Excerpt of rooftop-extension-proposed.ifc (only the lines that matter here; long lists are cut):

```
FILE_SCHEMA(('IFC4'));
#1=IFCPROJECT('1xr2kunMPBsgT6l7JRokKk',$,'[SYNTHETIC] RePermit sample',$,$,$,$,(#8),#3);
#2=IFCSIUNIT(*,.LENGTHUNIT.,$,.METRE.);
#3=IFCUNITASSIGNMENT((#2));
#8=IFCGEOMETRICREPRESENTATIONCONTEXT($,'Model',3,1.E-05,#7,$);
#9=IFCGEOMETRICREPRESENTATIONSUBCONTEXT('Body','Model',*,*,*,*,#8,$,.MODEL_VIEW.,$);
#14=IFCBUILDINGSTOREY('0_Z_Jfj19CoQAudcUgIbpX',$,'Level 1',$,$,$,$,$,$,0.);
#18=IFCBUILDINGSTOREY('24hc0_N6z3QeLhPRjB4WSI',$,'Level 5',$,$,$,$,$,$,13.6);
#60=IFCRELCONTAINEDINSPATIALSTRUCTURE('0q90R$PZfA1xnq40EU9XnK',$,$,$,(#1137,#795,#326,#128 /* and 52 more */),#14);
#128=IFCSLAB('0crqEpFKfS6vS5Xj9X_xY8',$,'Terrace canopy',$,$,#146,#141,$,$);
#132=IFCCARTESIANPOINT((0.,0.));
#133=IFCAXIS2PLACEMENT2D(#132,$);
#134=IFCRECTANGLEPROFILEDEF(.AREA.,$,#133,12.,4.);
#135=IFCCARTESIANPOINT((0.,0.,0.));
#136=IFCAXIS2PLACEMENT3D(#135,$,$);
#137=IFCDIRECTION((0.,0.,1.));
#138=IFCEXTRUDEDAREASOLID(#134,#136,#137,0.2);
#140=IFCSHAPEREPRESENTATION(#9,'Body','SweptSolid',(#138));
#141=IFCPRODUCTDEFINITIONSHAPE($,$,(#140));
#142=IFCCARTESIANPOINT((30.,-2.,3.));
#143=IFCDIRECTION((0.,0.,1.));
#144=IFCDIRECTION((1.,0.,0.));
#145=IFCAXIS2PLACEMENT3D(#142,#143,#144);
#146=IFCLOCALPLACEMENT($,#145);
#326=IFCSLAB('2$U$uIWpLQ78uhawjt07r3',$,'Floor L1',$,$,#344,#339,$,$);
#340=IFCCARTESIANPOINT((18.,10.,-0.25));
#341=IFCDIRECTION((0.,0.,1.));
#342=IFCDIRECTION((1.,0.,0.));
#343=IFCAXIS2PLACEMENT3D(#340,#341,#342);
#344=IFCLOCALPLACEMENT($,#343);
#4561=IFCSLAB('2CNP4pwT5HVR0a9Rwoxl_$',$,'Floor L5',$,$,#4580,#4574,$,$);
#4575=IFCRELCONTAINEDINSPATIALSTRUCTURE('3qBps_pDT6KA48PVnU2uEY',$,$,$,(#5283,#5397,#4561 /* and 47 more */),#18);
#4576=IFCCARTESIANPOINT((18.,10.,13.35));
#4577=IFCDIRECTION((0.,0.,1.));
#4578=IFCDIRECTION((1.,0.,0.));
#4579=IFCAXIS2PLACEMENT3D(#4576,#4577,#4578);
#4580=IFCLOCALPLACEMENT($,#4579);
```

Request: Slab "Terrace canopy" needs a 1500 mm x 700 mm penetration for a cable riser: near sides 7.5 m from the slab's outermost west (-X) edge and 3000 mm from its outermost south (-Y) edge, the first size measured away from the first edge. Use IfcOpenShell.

```python
import numpy as np
import ifcopenshell
import ifcopenshell.api.feature
import ifcopenshell.api.geometry
import ifcopenshell.api.root
import ifcopenshell.geom
import ifcopenshell.util.placement
import ifcopenshell.util.representation
import ifcopenshell.util.shape
import ifcopenshell.util.unit

model = ifcopenshell.open("rooftop-extension-proposed.ifc")
unit_scale = ifcopenshell.util.unit.calculate_unit_scale(model)
settings = ifcopenshell.geom.settings()


def volume(element):
    """Net volume in cubic metres, openings subtracted."""
    shape = ifcopenshell.geom.create_shape(settings, element)
    return ifcopenshell.util.shape.get_volume(shape.geometry)


slab = model.by_guid("0crqEpFKfS6vS5Xj9X_xY8")
before = volume(slab)

# Extent in the slab's own axes, in metres. The edges named are its -X and -Y sides.
slab_shape = ifcopenshell.geom.create_shape(settings, slab)
vertices = ifcopenshell.util.shape.get_vertices(slab_shape.geometry)
x_min, y_min, bottom = vertices.min(axis=0)
top = vertices[:, 2].max()

opening = ifcopenshell.api.root.create_entity(model, ifc_class="IfcOpeningElement", name="Cable riser opening", predefined_type="OPENING")
context = ifcopenshell.util.representation.get_context(model, "Model", "Body", "MODEL_VIEW")
width, depth = 1.5, 0.7
outline = [(0.0, 0.0), (width, 0.0), (width, depth), (0.0, depth), (0.0, 0.0)]
# Overshoot both faces by 50 mm so the cut is clean.
shape = ifcopenshell.api.geometry.add_slab_representation(
    model, context=context, depth=top - bottom + 0.1, polyline=outline
)
ifcopenshell.api.geometry.assign_representation(model, product=opening, representation=shape)

matrix = ifcopenshell.util.placement.get_local_placement(slab.ObjectPlacement)
matrix[:, 3] = matrix @ np.append(np.array([x_min + 7.5, y_min + 3, bottom - 0.05]) / unit_scale, 1.0)
ifcopenshell.api.geometry.edit_object_placement(model, product=opening, matrix=matrix, is_si=False)
ifcopenshell.api.feature.add_feature(model, feature=opening, element=slab)

after = volume(slab)

print(f"slab volume {before:.3f} -> {after:.3f} m3")

model.write("rooftop-extension-proposed_edited.ifc")
```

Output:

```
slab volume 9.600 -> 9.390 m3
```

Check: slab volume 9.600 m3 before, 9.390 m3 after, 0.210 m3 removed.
